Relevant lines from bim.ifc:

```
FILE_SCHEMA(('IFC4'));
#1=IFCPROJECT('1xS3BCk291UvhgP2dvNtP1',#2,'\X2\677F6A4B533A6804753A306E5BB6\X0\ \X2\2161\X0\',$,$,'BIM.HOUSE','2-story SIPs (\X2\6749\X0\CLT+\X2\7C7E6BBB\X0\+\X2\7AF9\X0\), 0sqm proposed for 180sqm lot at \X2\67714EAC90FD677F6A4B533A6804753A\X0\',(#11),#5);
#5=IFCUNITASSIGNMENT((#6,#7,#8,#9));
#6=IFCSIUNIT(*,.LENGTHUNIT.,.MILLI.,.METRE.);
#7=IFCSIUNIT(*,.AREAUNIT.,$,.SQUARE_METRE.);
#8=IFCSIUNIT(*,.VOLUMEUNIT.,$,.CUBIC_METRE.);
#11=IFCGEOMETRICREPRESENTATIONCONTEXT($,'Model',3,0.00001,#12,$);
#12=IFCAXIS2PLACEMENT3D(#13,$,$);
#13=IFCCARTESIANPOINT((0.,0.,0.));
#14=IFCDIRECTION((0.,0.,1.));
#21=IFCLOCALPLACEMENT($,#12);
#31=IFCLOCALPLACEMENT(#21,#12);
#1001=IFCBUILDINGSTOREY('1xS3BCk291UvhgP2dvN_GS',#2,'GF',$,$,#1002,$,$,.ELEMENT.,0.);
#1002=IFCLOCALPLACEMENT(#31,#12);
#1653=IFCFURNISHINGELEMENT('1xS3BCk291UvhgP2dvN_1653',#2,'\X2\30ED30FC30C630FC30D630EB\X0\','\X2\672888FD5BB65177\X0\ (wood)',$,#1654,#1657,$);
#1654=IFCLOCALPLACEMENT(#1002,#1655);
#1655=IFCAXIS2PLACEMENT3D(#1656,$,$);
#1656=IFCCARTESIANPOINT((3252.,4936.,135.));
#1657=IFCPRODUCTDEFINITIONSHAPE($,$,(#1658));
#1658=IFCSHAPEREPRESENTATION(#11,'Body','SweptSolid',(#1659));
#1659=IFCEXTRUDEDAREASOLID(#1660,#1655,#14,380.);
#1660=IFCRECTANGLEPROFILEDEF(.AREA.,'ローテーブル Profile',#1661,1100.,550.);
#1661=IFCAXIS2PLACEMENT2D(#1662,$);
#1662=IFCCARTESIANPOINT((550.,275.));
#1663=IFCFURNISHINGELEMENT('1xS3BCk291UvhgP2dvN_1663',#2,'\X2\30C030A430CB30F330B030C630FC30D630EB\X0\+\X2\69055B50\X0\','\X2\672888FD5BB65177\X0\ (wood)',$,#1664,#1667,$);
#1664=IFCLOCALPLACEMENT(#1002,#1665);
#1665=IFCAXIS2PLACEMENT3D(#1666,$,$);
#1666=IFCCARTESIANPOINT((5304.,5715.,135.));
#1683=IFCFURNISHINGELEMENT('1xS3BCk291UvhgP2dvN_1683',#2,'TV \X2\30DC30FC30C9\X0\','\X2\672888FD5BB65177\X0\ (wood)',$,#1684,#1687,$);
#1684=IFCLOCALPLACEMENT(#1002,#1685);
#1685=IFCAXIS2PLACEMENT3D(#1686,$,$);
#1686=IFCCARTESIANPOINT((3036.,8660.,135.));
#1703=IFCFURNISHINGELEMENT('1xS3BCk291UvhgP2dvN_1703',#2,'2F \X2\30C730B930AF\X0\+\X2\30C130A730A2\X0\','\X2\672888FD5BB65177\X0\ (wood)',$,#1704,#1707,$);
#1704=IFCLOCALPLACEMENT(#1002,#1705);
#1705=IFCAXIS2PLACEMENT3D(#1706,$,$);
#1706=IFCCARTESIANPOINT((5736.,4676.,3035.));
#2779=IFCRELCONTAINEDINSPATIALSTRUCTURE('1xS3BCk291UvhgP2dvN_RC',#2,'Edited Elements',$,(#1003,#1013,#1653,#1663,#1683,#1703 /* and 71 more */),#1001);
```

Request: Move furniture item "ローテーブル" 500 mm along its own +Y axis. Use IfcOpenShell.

```python
import ifcopenshell
import ifcopenshell.api.geometry
import ifcopenshell.util.placement

model = ifcopenshell.open("bim.ifc")

item = model.by_guid("1xS3BCk291UvhgP2dvN_1653")
matrix = ifcopenshell.util.placement.get_local_placement(item.ObjectPlacement)
matrix[:3, 3] += matrix[:3, 1] * 500.0
ifcopenshell.api.geometry.edit_object_placement(model, product=item, matrix=matrix, is_si=False)

print(ifcopenshell.util.placement.get_local_placement(item.ObjectPlacement).round(3) + 0.0)

model.write("bim_edited.ifc")
```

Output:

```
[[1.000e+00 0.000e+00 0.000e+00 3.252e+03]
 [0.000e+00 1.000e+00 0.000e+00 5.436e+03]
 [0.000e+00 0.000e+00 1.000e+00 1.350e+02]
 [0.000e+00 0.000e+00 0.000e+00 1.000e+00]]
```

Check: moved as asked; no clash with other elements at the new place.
